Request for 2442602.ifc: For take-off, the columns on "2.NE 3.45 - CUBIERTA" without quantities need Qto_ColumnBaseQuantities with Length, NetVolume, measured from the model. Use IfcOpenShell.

First a look at what the model holds.

```python
import ifcopenshell
import ifcopenshell.util.element
import ifcopenshell.util.unit

model = ifcopenshell.open("2442602.ifc")
print(model.schema)
for unit_type in ("LENGTHUNIT", "AREAUNIT", "VOLUMEUNIT"):
    print(unit_type, ifcopenshell.util.unit.calculate_unit_scale(model, unit_type))
storey = next(s for s in model.by_type("IfcBuildingStorey") if s.Name == "2.NE 3.45 - CUBIERTA")
columns = [e for e in ifcopenshell.util.element.get_decomposition(storey) if e.is_a("IfcColumn")]
for e in sorted(columns, key=lambda e: e.id()):
    print(e.id(), e.is_a(), e.Name, list(ifcopenshell.util.element.get_psets(e, qtos_only=True)), sep=" | ")
```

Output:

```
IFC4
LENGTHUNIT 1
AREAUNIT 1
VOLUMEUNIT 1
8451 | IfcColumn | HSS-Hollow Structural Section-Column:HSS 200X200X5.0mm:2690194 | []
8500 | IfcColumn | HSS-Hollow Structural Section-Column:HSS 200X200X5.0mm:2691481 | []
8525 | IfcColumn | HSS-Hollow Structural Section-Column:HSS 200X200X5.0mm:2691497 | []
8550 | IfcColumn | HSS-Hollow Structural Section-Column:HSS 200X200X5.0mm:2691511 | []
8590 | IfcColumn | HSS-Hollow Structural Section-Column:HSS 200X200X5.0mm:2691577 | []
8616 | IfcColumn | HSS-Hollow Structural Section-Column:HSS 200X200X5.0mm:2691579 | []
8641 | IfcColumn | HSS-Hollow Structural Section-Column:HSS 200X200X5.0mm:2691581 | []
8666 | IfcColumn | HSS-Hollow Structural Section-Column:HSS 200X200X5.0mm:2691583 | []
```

```python
import ifcopenshell
import ifcopenshell.api.pset
import ifcopenshell.geom
import ifcopenshell.util.element
import ifcopenshell.util.shape
import ifcopenshell.util.unit

model = ifcopenshell.open("2442602.ifc")
unit_scale = ifcopenshell.util.unit.calculate_unit_scale(model)
volume_scale = ifcopenshell.util.unit.calculate_unit_scale(model, "VOLUMEUNIT")
settings = ifcopenshell.geom.settings()

storey = next(s for s in model.by_type("IfcBuildingStorey") if s.Name == "2.NE 3.45 - CUBIERTA")
columns = [e for e in ifcopenshell.util.element.get_decomposition(storey) if e.is_a("IfcColumn")]

for e in sorted(columns, key=lambda e: e.id()):
    if ifcopenshell.util.element.get_psets(e, qtos_only=True, should_inherit=False):
        continue
    # Geometry comes back in metres, in the element's own axes.
    shape = ifcopenshell.geom.create_shape(settings, e)
    values = {
        "Length": ifcopenshell.util.shape.get_z(shape.geometry) / unit_scale,
        "NetVolume": ifcopenshell.util.shape.get_volume(shape.geometry) / volume_scale,
    }
    qto = ifcopenshell.api.pset.add_qto(model, product=e, name="Qto_ColumnBaseQuantities")
    ifcopenshell.api.pset.edit_qto(model, qto=qto, properties=values)
    print(e.id(), {k: round(v, 3) for k, v in values.items()})

model.write("2442602_rev.ifc")
```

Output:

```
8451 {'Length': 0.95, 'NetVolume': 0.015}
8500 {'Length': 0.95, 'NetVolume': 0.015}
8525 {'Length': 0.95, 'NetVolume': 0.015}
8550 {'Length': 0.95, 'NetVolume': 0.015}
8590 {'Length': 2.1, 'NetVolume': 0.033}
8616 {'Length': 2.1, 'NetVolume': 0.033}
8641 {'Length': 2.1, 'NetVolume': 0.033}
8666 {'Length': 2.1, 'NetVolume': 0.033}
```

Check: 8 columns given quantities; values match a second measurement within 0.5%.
